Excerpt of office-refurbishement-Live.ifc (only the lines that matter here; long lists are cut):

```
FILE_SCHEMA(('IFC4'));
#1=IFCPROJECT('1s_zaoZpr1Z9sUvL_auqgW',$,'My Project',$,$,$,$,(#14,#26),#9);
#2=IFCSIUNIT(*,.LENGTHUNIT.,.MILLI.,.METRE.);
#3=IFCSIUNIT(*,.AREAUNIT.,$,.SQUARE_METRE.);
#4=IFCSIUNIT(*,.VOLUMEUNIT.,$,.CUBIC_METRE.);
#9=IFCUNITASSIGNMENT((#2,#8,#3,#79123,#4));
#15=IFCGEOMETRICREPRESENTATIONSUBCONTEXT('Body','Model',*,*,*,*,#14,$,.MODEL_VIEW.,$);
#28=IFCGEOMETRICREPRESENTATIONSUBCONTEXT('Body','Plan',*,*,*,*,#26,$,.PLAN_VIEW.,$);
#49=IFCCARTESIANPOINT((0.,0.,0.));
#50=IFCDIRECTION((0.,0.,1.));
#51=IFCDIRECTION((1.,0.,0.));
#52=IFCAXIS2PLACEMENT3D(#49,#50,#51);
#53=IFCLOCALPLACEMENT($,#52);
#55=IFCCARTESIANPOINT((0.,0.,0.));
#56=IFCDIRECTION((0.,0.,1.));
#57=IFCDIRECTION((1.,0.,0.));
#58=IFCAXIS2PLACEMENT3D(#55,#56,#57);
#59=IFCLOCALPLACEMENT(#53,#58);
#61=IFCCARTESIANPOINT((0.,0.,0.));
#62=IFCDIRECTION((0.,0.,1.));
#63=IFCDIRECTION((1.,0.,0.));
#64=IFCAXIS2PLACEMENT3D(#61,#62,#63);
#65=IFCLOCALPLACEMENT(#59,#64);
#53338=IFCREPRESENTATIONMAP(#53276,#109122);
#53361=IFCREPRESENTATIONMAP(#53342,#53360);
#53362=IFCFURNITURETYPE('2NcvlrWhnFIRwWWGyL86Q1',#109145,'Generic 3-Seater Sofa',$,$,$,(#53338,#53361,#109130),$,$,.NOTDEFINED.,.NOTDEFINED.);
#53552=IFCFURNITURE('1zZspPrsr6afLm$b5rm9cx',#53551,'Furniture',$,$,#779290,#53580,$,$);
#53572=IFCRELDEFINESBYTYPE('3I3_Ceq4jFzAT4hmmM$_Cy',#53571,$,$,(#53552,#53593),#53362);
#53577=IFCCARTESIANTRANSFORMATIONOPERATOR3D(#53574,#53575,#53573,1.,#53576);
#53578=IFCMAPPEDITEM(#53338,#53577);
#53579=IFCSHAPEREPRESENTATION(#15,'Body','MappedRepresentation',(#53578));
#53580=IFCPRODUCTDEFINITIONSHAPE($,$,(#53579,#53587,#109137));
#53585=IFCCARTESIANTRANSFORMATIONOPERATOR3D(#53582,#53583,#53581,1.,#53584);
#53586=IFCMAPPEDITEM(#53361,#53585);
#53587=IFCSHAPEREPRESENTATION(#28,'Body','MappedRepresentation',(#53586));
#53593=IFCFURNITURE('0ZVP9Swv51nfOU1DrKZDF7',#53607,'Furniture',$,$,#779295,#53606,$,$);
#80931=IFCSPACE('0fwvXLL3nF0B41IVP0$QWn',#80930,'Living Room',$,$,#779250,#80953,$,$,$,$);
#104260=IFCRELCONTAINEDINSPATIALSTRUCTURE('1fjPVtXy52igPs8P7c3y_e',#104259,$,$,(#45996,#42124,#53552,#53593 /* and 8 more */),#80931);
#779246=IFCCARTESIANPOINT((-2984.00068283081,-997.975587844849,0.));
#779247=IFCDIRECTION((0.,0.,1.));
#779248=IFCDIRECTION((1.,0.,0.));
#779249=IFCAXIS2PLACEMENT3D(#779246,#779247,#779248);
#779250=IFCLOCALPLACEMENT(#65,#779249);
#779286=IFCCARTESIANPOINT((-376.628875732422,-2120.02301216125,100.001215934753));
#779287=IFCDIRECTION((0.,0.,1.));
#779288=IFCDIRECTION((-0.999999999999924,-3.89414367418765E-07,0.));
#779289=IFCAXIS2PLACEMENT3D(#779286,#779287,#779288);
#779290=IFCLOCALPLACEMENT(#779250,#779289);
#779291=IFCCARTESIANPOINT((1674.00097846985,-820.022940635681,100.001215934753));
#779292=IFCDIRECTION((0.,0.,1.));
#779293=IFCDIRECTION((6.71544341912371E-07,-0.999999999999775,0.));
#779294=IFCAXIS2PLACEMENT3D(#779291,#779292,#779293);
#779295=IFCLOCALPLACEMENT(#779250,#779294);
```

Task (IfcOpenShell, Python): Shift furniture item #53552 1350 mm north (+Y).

```python
import ifcopenshell
import ifcopenshell.api.geometry
import ifcopenshell.util.placement

model = ifcopenshell.open("office-refurbishement-Live.ifc")

item = model.by_guid("1zZspPrsr6afLm$b5rm9cx")
matrix = ifcopenshell.util.placement.get_local_placement(item.ObjectPlacement)
matrix[1, 3] += 1350.0
ifcopenshell.api.geometry.edit_object_placement(model, product=item, matrix=matrix, is_si=False)

print(ifcopenshell.util.placement.get_local_placement(item.ObjectPlacement).round(3) + 0.0)

model.write("office-refurbishement-Live_edited.ifc")
```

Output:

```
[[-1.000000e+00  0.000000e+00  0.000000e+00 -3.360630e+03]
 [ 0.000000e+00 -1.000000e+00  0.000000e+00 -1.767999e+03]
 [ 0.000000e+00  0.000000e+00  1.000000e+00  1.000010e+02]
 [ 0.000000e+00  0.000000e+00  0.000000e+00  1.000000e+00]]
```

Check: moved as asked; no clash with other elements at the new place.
